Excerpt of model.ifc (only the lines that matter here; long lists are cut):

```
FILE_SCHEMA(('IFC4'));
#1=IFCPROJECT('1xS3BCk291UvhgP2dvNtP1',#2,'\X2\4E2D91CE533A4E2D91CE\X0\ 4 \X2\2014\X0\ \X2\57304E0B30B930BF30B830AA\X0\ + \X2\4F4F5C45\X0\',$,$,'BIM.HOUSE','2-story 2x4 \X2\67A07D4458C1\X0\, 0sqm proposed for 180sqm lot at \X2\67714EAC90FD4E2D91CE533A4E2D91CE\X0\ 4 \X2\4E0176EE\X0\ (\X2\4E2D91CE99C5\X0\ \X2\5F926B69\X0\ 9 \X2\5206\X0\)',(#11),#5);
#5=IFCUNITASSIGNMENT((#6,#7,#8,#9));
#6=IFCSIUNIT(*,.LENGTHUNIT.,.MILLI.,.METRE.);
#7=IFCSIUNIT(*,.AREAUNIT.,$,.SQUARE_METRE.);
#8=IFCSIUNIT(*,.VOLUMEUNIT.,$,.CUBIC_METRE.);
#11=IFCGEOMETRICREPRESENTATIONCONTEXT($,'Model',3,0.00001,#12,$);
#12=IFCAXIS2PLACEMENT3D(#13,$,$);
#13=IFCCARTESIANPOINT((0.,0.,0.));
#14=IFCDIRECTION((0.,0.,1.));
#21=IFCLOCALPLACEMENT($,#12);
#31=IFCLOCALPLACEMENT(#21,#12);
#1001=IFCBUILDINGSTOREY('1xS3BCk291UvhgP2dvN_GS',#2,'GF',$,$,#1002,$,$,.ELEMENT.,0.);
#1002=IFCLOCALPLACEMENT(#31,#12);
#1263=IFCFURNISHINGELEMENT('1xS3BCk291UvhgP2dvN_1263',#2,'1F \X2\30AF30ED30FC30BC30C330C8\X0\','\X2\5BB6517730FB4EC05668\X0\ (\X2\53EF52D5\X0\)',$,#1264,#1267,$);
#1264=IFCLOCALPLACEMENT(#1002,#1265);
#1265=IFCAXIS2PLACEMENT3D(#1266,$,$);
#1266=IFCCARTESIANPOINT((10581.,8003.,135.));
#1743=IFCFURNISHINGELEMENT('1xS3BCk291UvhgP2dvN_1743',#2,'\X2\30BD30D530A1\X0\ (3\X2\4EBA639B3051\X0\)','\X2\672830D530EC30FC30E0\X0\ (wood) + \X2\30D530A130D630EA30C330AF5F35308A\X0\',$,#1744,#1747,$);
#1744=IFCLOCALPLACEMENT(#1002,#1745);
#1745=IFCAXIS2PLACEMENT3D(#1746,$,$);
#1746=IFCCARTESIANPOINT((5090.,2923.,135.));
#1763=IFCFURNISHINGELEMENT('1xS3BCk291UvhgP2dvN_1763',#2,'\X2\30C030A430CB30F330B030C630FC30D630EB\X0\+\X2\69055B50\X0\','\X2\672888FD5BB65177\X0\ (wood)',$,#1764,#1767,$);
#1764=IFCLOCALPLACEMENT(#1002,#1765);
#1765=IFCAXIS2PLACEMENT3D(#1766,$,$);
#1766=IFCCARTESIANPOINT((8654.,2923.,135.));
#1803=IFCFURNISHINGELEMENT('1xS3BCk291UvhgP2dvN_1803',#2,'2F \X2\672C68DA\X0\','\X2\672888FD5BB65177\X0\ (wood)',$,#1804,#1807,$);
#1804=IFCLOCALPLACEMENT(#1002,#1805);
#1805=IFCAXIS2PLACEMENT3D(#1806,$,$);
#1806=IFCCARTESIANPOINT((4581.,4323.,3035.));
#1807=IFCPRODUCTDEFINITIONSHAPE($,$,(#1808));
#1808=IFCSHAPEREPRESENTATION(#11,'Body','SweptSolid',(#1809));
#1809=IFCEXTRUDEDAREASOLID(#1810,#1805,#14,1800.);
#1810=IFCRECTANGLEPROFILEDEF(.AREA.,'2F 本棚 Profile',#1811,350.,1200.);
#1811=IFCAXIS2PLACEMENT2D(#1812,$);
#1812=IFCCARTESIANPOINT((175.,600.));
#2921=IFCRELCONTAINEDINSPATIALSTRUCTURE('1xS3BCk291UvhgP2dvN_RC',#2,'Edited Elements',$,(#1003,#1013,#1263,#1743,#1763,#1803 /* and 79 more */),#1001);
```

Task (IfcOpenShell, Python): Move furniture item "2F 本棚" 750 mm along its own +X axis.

```python
import ifcopenshell
import ifcopenshell.api.geometry
import ifcopenshell.util.placement

model = ifcopenshell.open("model.ifc")

item = model.by_guid("1xS3BCk291UvhgP2dvN_1803")
matrix = ifcopenshell.util.placement.get_local_placement(item.ObjectPlacement)
matrix[:3, 3] += matrix[:3, 0] * 750.0
ifcopenshell.api.geometry.edit_object_placement(model, product=item, matrix=matrix, is_si=False)

print(ifcopenshell.util.placement.get_local_placement(item.ObjectPlacement).round(3) + 0.0)

model.write("model_rev.ifc")
```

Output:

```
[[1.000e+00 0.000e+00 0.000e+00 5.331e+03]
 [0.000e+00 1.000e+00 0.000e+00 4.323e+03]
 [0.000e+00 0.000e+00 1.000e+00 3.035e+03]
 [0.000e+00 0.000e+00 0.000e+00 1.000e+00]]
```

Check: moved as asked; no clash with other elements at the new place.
